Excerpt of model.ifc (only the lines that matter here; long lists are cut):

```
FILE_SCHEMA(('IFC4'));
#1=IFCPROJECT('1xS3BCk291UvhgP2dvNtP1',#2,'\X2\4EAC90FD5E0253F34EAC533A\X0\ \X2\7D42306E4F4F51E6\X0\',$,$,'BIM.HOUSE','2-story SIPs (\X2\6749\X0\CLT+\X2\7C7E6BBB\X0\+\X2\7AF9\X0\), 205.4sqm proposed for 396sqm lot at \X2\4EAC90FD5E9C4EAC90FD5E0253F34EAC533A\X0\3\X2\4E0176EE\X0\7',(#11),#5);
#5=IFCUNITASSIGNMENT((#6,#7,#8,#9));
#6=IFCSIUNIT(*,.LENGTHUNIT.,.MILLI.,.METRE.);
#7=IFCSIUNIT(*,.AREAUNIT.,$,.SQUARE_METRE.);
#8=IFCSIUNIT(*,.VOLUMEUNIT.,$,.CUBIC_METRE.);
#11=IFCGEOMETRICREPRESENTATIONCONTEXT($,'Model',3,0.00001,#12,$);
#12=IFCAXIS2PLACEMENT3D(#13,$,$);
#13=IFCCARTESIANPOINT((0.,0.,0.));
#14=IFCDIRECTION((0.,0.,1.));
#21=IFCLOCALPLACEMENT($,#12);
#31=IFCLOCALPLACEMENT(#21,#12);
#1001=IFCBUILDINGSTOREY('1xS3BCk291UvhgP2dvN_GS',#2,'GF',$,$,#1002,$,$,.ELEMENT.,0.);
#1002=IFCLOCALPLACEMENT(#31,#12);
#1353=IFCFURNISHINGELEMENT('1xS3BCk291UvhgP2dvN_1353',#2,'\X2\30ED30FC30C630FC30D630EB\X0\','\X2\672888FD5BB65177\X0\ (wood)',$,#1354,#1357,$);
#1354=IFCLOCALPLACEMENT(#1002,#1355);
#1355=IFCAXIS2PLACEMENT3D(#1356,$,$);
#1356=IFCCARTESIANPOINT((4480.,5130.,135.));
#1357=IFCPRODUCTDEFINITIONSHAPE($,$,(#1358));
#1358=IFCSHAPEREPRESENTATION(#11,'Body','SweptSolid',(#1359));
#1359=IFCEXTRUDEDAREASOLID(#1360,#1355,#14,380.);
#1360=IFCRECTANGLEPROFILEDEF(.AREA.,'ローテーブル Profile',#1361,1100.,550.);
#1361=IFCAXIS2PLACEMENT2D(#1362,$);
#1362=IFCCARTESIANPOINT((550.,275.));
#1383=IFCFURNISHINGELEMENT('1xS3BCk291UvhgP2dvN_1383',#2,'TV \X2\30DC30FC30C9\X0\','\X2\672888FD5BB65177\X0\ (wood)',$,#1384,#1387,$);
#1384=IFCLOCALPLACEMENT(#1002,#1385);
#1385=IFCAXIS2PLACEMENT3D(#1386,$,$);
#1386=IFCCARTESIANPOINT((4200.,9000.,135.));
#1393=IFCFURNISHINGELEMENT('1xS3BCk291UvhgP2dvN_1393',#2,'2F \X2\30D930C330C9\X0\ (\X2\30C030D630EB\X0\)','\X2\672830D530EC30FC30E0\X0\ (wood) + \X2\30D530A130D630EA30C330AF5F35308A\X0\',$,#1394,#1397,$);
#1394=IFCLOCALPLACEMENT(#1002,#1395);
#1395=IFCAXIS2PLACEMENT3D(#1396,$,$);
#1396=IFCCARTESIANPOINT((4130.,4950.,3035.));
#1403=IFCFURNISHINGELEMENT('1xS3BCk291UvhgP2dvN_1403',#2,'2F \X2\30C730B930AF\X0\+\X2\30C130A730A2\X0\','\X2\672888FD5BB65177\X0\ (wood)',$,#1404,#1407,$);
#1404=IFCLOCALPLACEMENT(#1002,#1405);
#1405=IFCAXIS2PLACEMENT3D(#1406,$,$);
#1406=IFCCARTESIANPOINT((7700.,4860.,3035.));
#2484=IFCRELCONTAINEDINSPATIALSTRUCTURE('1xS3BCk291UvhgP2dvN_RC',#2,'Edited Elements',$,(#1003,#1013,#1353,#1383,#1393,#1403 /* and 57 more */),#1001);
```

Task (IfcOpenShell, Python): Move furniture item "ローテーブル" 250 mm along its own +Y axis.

```python
import ifcopenshell
import ifcopenshell.api.geometry
import ifcopenshell.util.placement
import ifcopenshell.util.unit

model = ifcopenshell.open("model.ifc")
unit_scale = ifcopenshell.util.unit.calculate_unit_scale(model)

item = model.by_guid("1xS3BCk291UvhgP2dvN_1353")
matrix = ifcopenshell.util.placement.get_local_placement(item.ObjectPlacement)
matrix[:3, 3] += matrix[:3, 1] * 0.25 / unit_scale
ifcopenshell.api.geometry.edit_object_placement(model, product=item, matrix=matrix, is_si=False)

print(ifcopenshell.util.placement.get_local_placement(item.ObjectPlacement).round(3) + 0.0)

model.write("model_edited.ifc")
```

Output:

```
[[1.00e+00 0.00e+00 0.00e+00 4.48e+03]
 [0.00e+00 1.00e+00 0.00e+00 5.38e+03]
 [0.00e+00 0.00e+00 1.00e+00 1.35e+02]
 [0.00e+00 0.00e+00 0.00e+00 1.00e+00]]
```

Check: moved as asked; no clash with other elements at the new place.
